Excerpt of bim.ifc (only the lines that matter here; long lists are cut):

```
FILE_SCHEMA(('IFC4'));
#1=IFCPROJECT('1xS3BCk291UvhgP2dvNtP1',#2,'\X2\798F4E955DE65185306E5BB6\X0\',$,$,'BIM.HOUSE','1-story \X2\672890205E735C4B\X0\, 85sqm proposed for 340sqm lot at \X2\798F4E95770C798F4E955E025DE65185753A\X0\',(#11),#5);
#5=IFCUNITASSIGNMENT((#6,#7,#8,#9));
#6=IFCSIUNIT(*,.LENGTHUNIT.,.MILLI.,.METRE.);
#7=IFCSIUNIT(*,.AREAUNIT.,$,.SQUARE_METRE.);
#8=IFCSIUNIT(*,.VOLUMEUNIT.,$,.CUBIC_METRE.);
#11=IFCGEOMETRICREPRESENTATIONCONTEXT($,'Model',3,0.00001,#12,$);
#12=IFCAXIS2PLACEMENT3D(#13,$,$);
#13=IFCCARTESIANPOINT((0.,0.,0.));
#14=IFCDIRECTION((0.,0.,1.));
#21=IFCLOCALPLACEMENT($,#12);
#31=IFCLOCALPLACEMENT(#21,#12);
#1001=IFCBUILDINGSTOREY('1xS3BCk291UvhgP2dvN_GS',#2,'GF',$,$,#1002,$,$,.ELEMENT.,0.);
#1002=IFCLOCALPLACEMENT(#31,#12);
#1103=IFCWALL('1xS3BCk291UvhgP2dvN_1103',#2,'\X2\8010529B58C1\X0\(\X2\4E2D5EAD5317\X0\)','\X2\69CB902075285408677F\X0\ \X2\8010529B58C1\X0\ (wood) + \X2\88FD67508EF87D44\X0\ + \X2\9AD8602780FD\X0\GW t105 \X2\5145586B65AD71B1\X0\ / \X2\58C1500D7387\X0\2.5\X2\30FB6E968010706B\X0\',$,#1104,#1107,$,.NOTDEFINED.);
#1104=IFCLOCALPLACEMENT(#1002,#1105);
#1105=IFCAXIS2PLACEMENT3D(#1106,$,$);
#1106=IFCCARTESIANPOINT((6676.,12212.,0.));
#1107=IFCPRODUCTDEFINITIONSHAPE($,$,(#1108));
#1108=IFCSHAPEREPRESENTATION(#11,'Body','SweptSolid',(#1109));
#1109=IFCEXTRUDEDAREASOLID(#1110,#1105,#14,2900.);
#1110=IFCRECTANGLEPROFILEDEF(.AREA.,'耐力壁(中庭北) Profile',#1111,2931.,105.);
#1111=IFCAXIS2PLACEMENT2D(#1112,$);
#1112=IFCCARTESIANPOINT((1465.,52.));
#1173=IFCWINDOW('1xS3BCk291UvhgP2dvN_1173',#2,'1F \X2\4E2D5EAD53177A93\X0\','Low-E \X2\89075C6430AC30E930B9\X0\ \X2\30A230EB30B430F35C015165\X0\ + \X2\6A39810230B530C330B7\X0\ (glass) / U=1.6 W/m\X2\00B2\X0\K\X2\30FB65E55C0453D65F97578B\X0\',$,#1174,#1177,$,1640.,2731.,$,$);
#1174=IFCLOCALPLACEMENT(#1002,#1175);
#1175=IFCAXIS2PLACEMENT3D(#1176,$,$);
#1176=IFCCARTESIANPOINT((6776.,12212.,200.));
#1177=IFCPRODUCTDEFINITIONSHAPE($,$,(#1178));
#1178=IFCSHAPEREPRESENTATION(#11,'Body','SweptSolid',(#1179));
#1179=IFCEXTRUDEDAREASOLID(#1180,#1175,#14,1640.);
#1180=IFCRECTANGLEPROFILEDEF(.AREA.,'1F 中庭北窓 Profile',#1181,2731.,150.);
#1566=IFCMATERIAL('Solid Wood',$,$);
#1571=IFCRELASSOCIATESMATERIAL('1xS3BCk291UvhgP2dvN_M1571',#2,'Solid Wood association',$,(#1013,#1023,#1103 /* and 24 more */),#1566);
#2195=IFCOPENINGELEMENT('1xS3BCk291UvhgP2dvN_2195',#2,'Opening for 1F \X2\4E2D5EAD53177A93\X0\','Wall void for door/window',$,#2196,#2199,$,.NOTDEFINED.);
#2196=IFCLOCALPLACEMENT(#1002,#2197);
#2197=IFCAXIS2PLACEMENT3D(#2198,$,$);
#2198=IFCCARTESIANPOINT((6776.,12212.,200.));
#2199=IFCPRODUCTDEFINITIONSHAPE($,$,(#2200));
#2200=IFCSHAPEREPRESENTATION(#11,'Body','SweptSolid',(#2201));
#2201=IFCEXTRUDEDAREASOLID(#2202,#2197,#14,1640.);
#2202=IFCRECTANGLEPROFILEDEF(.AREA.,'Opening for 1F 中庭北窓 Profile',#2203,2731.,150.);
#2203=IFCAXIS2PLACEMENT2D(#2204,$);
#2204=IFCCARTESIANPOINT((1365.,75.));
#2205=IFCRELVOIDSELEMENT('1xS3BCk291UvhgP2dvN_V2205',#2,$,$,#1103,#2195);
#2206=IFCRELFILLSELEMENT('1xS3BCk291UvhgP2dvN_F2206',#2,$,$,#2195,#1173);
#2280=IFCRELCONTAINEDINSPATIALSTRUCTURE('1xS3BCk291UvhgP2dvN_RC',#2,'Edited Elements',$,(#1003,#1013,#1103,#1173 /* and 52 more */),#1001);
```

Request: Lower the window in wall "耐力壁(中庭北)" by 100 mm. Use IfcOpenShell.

```python
import numpy as np
import ifcopenshell
import ifcopenshell.api.geometry
import ifcopenshell.util.placement
import ifcopenshell.util.unit

model = ifcopenshell.open("bim.ifc")
unit_scale = ifcopenshell.util.unit.calculate_unit_scale(model)

window = model.by_guid("1xS3BCk291UvhgP2dvN_1173")
opening = window.FillsVoids[0].RelatingOpeningElement
dz = -0.1 / unit_scale

shift = np.array([0.0, 0.0, dz])
# The window is not placed relative to its opening, so move both.
for product in (opening, window):
    matrix = ifcopenshell.util.placement.get_local_placement(product.ObjectPlacement)
    matrix[:3, 3] += shift
    ifcopenshell.api.geometry.edit_object_placement(model, product=product, matrix=matrix, is_si=False)

print(f"moved by {dz * unit_scale:+.3f} m")

model.write("bim_edited.ifc")
```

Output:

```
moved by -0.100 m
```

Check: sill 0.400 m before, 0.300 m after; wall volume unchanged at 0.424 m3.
